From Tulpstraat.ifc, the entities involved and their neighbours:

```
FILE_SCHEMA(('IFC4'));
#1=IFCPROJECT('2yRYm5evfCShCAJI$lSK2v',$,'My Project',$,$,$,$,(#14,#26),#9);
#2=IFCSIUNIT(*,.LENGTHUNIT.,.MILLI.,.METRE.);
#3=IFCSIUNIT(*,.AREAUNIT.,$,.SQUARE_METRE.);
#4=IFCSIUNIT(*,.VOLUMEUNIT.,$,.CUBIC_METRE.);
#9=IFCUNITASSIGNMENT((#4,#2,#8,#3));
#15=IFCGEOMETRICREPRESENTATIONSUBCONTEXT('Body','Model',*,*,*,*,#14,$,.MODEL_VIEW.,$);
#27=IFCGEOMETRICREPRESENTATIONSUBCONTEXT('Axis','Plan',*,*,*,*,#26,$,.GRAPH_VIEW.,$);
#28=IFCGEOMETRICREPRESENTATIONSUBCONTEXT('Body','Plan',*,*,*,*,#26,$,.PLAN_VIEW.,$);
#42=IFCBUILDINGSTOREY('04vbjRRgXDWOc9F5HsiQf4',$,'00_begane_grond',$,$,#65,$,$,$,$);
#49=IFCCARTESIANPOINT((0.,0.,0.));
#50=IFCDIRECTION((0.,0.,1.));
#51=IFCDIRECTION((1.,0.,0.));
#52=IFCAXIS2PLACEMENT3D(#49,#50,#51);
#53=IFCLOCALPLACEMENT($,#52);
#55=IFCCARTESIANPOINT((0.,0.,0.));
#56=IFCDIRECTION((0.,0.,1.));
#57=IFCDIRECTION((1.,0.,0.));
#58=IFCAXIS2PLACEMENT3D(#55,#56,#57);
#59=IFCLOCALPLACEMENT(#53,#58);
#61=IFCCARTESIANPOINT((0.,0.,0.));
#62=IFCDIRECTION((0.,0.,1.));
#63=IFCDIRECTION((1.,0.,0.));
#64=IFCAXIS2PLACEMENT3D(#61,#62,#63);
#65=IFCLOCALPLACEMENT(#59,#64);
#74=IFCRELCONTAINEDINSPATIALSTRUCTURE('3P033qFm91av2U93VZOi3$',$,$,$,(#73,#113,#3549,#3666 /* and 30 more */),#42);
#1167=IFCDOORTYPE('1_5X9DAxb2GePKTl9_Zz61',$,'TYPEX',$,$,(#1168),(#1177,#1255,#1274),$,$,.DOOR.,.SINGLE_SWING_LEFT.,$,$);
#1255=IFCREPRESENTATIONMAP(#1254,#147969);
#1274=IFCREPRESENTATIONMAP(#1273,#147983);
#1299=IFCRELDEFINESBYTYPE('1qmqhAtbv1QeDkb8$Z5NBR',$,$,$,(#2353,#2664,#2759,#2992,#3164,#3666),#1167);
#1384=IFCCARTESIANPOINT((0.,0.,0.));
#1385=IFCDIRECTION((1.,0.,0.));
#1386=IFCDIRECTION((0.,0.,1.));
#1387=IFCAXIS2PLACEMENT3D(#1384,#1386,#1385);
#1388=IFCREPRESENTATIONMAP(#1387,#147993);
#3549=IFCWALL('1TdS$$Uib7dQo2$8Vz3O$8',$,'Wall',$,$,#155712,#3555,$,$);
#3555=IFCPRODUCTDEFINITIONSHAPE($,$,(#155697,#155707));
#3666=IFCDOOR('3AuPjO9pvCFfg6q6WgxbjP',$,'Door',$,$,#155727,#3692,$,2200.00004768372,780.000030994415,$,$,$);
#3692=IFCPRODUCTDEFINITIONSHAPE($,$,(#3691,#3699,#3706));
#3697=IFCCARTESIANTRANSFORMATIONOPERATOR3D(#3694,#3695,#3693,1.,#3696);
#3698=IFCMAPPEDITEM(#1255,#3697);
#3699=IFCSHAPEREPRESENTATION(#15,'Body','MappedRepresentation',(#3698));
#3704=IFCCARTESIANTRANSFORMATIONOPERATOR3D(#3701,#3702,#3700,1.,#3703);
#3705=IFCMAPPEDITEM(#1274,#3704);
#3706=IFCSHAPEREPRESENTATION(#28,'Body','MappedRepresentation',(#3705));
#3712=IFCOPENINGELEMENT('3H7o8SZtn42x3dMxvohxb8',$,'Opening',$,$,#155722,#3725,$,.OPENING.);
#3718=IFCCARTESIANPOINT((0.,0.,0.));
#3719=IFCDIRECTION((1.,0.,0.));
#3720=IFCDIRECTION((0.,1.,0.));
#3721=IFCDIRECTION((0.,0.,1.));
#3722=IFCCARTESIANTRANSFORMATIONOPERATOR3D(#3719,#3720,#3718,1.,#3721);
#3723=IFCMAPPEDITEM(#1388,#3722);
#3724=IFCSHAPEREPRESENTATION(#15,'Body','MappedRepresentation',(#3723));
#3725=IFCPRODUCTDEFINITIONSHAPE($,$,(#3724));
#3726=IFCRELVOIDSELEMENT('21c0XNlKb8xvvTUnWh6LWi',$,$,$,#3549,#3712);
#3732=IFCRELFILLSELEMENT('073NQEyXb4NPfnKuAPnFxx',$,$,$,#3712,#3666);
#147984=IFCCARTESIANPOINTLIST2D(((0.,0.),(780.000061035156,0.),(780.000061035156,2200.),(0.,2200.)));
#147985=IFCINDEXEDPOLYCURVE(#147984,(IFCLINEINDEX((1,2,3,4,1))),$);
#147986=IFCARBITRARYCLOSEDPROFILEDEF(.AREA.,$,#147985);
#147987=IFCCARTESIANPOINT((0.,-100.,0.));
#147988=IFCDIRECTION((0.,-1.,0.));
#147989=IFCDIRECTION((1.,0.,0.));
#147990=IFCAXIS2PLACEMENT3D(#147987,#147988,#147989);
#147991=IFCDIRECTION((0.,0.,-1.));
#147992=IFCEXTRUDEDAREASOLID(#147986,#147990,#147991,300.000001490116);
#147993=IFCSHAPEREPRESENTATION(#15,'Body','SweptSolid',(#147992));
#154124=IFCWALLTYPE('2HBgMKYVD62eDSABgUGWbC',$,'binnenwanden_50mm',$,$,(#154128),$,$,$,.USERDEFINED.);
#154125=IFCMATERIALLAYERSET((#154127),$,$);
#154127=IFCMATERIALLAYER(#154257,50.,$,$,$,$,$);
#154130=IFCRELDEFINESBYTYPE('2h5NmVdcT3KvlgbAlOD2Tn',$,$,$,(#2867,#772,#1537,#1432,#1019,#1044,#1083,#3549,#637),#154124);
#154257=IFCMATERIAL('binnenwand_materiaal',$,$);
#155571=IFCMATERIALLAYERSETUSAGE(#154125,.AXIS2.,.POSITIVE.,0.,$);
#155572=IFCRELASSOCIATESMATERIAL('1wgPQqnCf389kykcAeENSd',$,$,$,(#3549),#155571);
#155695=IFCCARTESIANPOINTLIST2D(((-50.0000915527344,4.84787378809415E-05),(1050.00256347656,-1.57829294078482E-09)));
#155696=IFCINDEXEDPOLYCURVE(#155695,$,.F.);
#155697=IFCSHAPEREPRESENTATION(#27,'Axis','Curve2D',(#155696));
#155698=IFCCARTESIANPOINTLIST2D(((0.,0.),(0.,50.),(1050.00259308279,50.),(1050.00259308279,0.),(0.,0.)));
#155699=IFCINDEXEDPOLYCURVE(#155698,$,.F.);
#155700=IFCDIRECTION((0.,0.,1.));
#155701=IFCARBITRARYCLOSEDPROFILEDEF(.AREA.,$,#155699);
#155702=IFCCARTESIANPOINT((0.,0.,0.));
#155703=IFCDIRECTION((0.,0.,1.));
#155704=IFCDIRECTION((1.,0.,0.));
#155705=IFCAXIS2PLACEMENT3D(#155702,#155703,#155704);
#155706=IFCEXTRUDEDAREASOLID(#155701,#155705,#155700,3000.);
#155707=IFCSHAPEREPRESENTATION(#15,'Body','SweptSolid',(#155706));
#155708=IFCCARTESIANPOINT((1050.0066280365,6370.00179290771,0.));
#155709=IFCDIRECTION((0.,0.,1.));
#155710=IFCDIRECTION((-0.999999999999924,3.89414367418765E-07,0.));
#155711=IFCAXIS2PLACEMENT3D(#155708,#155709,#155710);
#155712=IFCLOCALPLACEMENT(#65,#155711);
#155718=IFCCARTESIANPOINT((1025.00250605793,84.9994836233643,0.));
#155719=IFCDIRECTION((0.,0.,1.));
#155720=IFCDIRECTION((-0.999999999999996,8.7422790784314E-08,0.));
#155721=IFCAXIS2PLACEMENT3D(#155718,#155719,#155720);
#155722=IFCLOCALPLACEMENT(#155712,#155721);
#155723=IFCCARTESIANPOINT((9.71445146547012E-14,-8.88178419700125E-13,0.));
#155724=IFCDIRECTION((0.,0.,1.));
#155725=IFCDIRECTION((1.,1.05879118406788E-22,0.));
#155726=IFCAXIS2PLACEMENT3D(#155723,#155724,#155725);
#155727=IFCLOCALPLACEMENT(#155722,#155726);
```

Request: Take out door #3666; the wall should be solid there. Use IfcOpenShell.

```python
import ifcopenshell
import ifcopenshell.api.feature
import ifcopenshell.api.root
import ifcopenshell.geom
import ifcopenshell.util.shape

model = ifcopenshell.open("Tulpstraat.ifc")
settings = ifcopenshell.geom.settings()


def volume(element):
    """Net volume in cubic metres, openings subtracted."""
    shape = ifcopenshell.geom.create_shape(settings, element)
    return ifcopenshell.util.shape.get_volume(shape.geometry)


door = model.by_guid("3AuPjO9pvCFfg6q6WgxbjP")
opening = door.FillsVoids[0].RelatingOpeningElement
wall = opening.VoidsElements[0].RelatingBuildingElement
before = volume(wall)

ifcopenshell.api.root.remove_product(model, product=door)
ifcopenshell.api.feature.remove_feature(model, feature=opening)

after = volume(wall)

print(f"wall volume {before:.3f} -> {after:.3f} m3")

model.write("Tulpstraat_rev.ifc")
```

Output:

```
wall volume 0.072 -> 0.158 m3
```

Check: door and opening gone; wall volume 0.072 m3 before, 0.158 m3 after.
